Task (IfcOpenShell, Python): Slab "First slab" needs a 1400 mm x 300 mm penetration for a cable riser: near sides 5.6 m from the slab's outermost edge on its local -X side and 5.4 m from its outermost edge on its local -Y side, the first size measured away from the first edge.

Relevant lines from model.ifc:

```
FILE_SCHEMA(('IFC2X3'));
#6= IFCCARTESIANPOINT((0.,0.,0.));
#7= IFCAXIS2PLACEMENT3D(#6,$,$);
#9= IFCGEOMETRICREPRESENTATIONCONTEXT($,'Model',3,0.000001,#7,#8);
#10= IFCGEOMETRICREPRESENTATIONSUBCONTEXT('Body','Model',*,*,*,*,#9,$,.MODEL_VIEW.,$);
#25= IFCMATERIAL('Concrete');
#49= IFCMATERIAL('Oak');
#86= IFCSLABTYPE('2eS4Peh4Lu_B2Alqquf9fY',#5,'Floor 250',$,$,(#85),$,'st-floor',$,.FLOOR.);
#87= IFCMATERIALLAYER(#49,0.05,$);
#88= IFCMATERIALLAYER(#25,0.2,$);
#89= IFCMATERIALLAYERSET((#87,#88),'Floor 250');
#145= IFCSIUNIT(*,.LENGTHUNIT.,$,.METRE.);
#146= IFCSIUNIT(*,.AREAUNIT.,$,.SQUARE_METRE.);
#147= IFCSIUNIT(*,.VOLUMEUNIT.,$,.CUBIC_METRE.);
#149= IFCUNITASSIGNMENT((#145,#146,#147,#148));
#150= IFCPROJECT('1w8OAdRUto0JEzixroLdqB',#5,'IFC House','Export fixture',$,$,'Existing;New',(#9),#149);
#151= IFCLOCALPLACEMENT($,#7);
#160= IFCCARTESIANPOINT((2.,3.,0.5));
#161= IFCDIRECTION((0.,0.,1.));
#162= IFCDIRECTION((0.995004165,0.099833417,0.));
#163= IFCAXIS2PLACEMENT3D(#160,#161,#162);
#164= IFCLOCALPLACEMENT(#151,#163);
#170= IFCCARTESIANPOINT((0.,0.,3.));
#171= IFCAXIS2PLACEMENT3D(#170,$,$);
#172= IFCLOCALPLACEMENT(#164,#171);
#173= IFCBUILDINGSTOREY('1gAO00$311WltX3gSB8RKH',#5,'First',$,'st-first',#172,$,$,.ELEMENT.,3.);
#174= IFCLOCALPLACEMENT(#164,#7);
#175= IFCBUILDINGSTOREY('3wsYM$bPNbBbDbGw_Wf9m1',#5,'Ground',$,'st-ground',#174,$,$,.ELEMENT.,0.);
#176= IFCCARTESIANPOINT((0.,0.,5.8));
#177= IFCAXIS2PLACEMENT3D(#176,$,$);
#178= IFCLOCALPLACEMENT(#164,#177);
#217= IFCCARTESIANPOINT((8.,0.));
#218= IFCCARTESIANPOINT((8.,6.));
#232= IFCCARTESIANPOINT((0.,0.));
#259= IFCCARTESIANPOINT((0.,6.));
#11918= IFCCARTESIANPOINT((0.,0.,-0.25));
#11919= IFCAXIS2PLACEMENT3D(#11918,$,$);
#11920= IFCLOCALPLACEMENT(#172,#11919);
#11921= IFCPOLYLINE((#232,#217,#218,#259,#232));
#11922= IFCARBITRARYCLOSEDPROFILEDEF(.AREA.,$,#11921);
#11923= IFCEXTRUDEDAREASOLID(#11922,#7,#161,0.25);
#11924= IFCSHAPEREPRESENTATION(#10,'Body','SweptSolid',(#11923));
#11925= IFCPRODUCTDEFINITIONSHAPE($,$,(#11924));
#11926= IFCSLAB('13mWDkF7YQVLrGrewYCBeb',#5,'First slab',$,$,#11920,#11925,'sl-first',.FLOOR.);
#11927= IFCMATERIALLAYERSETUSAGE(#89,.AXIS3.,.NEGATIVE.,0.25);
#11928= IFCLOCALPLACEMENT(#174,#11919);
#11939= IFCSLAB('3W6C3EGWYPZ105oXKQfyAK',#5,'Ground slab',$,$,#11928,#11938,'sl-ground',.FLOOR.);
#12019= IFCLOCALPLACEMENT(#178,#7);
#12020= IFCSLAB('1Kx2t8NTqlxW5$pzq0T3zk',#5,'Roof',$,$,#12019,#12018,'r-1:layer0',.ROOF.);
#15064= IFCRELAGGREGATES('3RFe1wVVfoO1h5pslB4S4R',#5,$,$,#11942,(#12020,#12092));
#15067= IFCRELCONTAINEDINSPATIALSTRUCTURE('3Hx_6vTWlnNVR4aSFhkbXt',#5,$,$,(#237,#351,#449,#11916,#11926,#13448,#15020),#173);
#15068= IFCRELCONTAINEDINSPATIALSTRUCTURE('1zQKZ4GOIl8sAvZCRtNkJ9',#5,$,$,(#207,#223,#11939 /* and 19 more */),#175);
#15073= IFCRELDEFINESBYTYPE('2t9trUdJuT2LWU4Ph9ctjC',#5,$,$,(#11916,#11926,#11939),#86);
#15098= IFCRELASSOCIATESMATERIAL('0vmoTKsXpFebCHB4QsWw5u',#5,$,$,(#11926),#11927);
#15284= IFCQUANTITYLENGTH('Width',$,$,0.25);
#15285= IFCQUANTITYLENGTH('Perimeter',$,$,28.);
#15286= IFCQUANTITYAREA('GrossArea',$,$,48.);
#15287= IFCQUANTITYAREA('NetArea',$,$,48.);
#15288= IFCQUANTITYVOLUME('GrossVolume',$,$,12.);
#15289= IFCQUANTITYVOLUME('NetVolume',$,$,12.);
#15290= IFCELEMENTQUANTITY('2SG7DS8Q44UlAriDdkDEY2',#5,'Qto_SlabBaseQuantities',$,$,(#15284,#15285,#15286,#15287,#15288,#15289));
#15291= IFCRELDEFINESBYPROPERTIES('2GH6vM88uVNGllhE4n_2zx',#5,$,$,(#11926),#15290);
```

```python
import numpy as np
import ifcopenshell
import ifcopenshell.api.feature
import ifcopenshell.api.geometry
import ifcopenshell.api.pset
import ifcopenshell.api.root
import ifcopenshell.geom
import ifcopenshell.util.element
import ifcopenshell.util.placement
import ifcopenshell.util.representation
import ifcopenshell.util.shape
import ifcopenshell.util.unit

model = ifcopenshell.open("model.ifc")
unit_scale = ifcopenshell.util.unit.calculate_unit_scale(model)
area_scale = ifcopenshell.util.unit.calculate_unit_scale(model, "AREAUNIT")
volume_scale = ifcopenshell.util.unit.calculate_unit_scale(model, "VOLUMEUNIT")
settings = ifcopenshell.geom.settings()


def volume(element):
    """Net volume in cubic metres, openings subtracted."""
    shape = ifcopenshell.geom.create_shape(settings, element)
    return ifcopenshell.util.shape.get_volume(shape.geometry)


slab = model.by_guid("13mWDkF7YQVLrGrewYCBeb")
before = volume(slab)

# Extent in the slab's own axes, in metres. The edges named are its -X and -Y sides.
slab_shape = ifcopenshell.geom.create_shape(settings, slab)
vertices = ifcopenshell.util.shape.get_vertices(slab_shape.geometry)
x_min, y_min, bottom = vertices.min(axis=0)
top = vertices[:, 2].max()

opening = ifcopenshell.api.root.create_entity(model, ifc_class="IfcOpeningElement", name="Cable riser opening")
context = ifcopenshell.util.representation.get_context(model, "Model", "Body", "MODEL_VIEW")
width, depth = 1.4, 0.3
outline = [(0.0, 0.0), (width, 0.0), (width, depth), (0.0, depth), (0.0, 0.0)]
# Overshoot both faces by 50 mm so the cut is clean.
shape = ifcopenshell.api.geometry.add_slab_representation(
    model, context=context, depth=top - bottom + 0.1, polyline=outline
)
ifcopenshell.api.geometry.assign_representation(model, product=opening, representation=shape)

matrix = ifcopenshell.util.placement.get_local_placement(slab.ObjectPlacement)
matrix[:, 3] = matrix @ np.append(np.array([x_min + 5.6, y_min + 5.4, bottom - 0.05]) / unit_scale, 1.0)
ifcopenshell.api.geometry.edit_object_placement(model, product=opening, matrix=matrix, is_si=False)
ifcopenshell.api.feature.add_feature(model, feature=opening, element=slab)

after = volume(slab)

# Update the slab's stored quantities.
qto = model.by_id(ifcopenshell.util.element.get_pset(slab, "Qto_SlabBaseQuantities", should_inherit=False)["id"])
ifcopenshell.api.pset.edit_qto(model, qto=qto, properties={
    "NetArea": after / (top - bottom) / area_scale,
    "NetVolume": after / volume_scale,
})

print(f"slab volume {before:.3f} -> {after:.3f} m3")

model.write("model_rev.ifc")
```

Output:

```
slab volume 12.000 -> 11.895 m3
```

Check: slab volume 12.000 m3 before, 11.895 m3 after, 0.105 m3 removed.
